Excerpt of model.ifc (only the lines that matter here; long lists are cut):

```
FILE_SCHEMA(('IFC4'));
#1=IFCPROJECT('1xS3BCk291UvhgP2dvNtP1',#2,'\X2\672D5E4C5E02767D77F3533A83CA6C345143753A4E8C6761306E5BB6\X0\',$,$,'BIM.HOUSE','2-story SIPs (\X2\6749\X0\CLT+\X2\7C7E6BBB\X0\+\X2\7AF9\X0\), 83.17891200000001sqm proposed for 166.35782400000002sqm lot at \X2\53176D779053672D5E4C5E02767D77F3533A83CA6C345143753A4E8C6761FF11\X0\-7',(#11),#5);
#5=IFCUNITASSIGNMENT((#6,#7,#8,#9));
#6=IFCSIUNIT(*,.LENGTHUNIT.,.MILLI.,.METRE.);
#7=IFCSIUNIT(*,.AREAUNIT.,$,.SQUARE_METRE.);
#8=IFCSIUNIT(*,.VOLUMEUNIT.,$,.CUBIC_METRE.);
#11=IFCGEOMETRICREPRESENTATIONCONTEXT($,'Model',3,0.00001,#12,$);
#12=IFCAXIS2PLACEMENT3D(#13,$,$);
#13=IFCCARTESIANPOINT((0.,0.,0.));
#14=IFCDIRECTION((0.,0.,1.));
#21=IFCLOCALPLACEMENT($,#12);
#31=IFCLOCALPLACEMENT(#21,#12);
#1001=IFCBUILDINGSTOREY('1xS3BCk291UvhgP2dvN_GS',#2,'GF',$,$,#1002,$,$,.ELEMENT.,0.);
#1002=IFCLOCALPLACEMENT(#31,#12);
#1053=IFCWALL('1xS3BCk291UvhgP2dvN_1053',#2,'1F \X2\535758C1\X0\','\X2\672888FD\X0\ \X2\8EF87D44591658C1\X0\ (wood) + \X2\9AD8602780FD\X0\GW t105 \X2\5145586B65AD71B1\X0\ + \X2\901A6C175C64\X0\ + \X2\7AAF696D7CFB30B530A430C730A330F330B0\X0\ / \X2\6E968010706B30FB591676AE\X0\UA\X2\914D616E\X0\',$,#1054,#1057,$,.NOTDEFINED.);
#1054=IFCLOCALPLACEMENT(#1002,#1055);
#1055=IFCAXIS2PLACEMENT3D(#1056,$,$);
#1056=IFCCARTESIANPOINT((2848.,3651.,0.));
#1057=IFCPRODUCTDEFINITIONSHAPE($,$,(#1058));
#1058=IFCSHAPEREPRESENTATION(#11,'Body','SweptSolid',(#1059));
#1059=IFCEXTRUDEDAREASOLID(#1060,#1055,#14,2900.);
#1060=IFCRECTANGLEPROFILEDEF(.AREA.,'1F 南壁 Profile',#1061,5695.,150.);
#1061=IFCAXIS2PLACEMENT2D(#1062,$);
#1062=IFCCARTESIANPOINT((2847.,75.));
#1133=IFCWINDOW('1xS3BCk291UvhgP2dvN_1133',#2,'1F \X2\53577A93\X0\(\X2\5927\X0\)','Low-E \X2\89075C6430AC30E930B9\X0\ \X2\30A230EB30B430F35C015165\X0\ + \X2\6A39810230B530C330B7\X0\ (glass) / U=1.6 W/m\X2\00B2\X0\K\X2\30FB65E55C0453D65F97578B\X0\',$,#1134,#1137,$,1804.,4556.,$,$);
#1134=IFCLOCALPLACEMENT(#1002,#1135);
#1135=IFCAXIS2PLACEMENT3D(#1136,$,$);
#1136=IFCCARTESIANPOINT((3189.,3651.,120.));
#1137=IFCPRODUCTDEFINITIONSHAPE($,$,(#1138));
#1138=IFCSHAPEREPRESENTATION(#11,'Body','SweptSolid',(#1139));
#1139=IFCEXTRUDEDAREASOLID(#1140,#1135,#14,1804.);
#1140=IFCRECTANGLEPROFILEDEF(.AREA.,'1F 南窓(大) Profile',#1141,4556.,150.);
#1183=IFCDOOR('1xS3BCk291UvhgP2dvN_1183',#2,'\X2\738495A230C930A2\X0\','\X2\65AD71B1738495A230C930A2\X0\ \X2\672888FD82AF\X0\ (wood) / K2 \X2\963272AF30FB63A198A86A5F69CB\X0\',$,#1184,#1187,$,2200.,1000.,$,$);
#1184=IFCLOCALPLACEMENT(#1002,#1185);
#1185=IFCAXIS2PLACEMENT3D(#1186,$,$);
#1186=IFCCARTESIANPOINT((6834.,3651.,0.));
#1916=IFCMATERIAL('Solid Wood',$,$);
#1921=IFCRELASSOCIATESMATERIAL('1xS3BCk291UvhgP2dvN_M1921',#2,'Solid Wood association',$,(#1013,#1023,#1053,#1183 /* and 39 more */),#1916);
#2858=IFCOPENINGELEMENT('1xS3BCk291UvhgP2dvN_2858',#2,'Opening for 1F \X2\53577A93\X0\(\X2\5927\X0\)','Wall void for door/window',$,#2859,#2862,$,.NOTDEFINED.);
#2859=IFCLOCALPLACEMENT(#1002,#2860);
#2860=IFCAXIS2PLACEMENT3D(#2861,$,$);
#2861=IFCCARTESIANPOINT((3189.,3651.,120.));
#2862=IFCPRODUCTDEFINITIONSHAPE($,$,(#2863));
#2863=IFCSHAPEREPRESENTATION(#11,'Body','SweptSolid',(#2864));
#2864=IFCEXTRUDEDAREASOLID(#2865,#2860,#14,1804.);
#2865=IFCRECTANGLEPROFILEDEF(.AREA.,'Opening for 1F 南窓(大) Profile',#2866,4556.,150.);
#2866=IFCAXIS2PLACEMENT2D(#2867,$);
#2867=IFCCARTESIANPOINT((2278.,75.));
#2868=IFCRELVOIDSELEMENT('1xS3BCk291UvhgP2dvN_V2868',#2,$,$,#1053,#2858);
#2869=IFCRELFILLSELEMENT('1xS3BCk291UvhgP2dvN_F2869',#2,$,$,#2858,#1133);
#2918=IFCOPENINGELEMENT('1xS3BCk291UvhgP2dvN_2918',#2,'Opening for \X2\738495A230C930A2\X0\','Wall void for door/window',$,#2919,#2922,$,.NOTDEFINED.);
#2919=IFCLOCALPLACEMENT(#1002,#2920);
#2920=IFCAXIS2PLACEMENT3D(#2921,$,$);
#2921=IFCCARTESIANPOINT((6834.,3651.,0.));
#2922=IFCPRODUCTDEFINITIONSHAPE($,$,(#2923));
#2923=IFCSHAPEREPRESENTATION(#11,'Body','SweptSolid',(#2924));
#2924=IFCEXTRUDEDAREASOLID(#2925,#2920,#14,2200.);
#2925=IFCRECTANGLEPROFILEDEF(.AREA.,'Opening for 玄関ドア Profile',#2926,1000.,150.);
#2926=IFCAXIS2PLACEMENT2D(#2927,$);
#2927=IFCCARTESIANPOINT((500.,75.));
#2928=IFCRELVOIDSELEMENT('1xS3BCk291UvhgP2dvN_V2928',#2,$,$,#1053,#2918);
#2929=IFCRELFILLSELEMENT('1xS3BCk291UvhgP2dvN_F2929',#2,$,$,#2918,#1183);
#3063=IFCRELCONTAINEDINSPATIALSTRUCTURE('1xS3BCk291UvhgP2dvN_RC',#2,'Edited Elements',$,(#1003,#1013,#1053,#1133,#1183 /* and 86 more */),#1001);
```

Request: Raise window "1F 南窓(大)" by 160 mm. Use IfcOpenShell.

```python
import numpy as np
import ifcopenshell
import ifcopenshell.api.geometry
import ifcopenshell.util.placement
import ifcopenshell.util.unit

model = ifcopenshell.open("model.ifc")
unit_scale = ifcopenshell.util.unit.calculate_unit_scale(model)

window = model.by_guid("1xS3BCk291UvhgP2dvN_1133")
opening = window.FillsVoids[0].RelatingOpeningElement
dz = 0.16 / unit_scale

shift = np.array([0.0, 0.0, dz])
# The window is not placed relative to its opening, so move both.
for product in (opening, window):
    matrix = ifcopenshell.util.placement.get_local_placement(product.ObjectPlacement)
    matrix[:3, 3] += shift
    ifcopenshell.api.geometry.edit_object_placement(model, product=product, matrix=matrix, is_si=False)

print(f"moved by {dz * unit_scale:+.3f} m")

model.write("model_v2.ifc")
```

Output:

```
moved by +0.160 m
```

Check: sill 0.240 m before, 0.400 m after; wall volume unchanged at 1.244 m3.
